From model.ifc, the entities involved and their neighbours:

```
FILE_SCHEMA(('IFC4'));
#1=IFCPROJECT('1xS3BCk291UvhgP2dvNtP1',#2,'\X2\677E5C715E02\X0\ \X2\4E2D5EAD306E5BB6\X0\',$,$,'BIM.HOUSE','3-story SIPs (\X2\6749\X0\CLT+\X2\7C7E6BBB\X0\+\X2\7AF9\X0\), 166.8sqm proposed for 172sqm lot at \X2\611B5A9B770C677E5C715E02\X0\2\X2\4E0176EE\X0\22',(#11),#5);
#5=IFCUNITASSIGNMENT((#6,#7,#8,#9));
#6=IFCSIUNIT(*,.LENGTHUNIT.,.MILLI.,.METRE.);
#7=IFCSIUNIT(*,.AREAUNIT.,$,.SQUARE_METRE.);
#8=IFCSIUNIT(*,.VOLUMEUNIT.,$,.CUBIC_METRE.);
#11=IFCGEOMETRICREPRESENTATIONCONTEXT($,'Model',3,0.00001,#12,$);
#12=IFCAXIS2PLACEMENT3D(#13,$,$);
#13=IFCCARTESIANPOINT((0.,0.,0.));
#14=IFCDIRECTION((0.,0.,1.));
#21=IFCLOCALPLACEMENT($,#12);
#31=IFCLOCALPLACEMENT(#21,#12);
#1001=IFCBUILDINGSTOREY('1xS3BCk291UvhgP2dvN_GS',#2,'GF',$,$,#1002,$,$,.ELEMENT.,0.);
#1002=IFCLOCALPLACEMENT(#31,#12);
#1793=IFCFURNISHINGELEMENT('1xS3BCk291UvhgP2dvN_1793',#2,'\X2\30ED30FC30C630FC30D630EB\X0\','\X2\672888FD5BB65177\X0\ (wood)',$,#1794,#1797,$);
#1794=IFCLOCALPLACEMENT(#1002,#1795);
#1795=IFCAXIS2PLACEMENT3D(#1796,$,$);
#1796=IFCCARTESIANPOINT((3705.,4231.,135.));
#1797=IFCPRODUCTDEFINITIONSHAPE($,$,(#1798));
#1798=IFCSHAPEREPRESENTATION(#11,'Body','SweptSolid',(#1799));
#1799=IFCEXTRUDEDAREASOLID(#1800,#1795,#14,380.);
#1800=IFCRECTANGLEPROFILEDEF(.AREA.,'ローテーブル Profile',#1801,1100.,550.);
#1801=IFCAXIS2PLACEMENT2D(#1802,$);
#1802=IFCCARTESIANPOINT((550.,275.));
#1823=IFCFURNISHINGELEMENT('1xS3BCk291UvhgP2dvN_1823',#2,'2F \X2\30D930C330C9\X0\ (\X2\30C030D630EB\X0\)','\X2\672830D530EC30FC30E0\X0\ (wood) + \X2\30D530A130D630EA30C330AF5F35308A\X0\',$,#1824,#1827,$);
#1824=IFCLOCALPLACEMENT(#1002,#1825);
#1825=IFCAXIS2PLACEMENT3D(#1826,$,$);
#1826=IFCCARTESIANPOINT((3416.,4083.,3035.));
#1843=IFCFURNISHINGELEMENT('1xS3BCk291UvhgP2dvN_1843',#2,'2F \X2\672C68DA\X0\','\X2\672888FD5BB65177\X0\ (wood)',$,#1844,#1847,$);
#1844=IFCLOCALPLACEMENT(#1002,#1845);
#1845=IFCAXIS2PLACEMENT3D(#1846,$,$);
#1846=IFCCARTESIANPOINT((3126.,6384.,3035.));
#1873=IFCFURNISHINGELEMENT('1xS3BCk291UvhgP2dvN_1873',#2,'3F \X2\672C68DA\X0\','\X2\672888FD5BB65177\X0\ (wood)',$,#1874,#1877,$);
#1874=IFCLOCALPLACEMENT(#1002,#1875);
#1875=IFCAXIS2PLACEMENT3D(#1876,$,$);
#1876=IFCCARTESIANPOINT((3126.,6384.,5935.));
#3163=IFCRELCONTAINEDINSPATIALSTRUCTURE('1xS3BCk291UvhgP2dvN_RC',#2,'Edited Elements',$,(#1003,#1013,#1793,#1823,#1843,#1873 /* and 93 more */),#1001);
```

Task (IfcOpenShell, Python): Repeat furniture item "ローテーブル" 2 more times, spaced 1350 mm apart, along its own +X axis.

```python
import ifcopenshell
import ifcopenshell.api.geometry
import ifcopenshell.api.root
import ifcopenshell.util.element
import ifcopenshell.util.placement
import ifcopenshell.util.unit

model = ifcopenshell.open("model.ifc")
unit_scale = ifcopenshell.util.unit.calculate_unit_scale(model)


def reuse_history(source, copy):
    """copy_class also copies each property set's owner history, people and application; keep the originals."""
    for rel in copy.IsDefinedBy:
        if rel.is_a("IfcRelDefinesByProperties") and (history := rel.RelatingPropertyDefinition.OwnerHistory):
            rel.RelatingPropertyDefinition.OwnerHistory = source.OwnerHistory
            ifcopenshell.util.element.remove_deep2(model, history)


source = model.by_id(1793)
base = ifcopenshell.util.placement.get_local_placement(source.ObjectPlacement)
step = base[:3, 0] * 1.35 / unit_scale

for i in range(1, 3):
    copy = ifcopenshell.api.root.copy_class(model, product=source)
    copy.Representation = ifcopenshell.util.element.copy_deep(
        model, source.Representation, exclude=["IfcGeometricRepresentationContext", "IfcRepresentationMap"]
    )
    reuse_history(source, copy)
    matrix = base.copy()
    matrix[:3, 3] += i * step
    print("added at", matrix[:3, 3].round(3) + 0.0)
    ifcopenshell.api.geometry.edit_object_placement(model, product=copy, matrix=matrix, is_si=False)

model.write("model_rev.ifc")
```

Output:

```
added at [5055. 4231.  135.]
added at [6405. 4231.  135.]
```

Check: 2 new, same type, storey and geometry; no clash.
